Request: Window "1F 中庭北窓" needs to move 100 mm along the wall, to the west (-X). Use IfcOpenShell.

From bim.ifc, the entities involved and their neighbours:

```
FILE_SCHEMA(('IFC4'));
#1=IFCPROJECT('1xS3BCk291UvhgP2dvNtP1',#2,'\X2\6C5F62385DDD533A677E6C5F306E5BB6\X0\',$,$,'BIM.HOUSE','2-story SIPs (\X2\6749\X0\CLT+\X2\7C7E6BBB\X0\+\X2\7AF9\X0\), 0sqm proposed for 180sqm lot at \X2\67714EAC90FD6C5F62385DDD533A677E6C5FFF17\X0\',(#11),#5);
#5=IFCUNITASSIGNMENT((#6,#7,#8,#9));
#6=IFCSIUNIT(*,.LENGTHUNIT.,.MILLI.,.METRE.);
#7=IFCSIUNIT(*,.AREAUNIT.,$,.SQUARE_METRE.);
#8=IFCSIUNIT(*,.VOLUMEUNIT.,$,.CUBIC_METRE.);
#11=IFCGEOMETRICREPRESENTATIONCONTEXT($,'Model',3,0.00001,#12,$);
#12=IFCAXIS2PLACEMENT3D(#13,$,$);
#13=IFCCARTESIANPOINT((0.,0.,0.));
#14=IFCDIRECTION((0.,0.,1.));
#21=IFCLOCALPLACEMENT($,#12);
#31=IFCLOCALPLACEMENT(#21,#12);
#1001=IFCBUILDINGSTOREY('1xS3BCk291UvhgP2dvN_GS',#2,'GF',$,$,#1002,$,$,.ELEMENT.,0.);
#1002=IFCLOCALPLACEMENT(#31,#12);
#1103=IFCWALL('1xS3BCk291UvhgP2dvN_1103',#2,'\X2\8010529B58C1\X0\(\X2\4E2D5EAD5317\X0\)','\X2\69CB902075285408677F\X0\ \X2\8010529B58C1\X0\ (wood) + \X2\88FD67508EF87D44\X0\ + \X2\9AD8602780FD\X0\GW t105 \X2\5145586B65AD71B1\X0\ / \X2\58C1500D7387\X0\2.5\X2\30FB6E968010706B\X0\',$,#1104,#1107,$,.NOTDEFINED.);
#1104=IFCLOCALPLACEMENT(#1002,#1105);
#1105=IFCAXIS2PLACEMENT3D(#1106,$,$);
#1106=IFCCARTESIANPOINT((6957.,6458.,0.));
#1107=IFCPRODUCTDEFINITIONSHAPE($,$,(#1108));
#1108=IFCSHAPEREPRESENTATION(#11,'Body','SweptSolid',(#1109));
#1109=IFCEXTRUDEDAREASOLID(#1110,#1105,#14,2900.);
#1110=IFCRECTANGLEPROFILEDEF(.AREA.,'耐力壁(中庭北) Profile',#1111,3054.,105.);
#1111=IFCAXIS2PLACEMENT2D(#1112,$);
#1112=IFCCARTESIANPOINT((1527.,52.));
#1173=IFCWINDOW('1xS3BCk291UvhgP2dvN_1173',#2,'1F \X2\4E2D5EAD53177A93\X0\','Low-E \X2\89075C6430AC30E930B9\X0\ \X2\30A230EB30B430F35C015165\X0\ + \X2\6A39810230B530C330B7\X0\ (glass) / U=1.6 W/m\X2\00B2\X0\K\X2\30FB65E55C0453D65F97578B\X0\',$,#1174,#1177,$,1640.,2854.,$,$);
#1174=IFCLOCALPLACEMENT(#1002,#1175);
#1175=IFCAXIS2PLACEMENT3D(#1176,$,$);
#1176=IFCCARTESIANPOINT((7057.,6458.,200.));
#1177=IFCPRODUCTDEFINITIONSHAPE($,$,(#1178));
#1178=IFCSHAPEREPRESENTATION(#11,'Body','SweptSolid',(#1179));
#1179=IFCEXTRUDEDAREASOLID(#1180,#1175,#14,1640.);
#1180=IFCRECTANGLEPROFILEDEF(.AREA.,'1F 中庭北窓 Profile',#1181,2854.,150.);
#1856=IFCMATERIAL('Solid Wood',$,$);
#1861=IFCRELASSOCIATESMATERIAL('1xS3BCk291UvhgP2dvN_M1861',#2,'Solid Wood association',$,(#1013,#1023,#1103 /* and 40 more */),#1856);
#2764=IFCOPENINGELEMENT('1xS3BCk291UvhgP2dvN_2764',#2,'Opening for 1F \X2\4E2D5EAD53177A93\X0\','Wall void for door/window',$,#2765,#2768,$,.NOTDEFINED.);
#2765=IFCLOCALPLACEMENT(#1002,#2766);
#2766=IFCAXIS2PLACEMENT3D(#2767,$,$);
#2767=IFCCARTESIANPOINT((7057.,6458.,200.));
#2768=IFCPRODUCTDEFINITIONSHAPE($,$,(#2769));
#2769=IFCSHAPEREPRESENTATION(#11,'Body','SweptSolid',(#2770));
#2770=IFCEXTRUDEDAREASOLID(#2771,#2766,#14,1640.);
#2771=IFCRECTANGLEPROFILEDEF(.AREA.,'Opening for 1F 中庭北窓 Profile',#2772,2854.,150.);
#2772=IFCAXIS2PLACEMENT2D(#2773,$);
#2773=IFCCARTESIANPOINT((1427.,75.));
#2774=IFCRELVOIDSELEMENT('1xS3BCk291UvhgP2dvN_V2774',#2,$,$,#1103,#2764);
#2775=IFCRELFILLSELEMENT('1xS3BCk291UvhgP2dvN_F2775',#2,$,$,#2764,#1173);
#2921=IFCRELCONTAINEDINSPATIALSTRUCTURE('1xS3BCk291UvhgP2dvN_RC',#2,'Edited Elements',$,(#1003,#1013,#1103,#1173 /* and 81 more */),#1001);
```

```python
import ifcopenshell
import ifcopenshell.api.geometry
import ifcopenshell.util.placement

model = ifcopenshell.open("bim.ifc")

window = model.by_id(1173)
opening = window.FillsVoids[0].RelatingOpeningElement
wall = opening.VoidsElements[0].RelatingBuildingElement

wall_matrix = ifcopenshell.util.placement.get_local_placement(wall.ObjectPlacement)
shift = wall_matrix[:3, 0] * -100.0
before = ifcopenshell.util.placement.get_local_placement(window.ObjectPlacement)[:3, 3].copy()

# The window is not placed relative to its opening, so move both.
for product in (opening, window):
    matrix = ifcopenshell.util.placement.get_local_placement(product.ObjectPlacement)
    matrix[:3, 3] += shift
    ifcopenshell.api.geometry.edit_object_placement(model, product=product, matrix=matrix, is_si=False)

after = ifcopenshell.util.placement.get_local_placement(window.ObjectPlacement)[:3, 3]
print("window moved by", (after - before).round(3) + 0.0)

model.write("bim_rev.ifc")
```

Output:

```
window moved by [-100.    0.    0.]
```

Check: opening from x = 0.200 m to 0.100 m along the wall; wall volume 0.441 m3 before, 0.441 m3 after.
